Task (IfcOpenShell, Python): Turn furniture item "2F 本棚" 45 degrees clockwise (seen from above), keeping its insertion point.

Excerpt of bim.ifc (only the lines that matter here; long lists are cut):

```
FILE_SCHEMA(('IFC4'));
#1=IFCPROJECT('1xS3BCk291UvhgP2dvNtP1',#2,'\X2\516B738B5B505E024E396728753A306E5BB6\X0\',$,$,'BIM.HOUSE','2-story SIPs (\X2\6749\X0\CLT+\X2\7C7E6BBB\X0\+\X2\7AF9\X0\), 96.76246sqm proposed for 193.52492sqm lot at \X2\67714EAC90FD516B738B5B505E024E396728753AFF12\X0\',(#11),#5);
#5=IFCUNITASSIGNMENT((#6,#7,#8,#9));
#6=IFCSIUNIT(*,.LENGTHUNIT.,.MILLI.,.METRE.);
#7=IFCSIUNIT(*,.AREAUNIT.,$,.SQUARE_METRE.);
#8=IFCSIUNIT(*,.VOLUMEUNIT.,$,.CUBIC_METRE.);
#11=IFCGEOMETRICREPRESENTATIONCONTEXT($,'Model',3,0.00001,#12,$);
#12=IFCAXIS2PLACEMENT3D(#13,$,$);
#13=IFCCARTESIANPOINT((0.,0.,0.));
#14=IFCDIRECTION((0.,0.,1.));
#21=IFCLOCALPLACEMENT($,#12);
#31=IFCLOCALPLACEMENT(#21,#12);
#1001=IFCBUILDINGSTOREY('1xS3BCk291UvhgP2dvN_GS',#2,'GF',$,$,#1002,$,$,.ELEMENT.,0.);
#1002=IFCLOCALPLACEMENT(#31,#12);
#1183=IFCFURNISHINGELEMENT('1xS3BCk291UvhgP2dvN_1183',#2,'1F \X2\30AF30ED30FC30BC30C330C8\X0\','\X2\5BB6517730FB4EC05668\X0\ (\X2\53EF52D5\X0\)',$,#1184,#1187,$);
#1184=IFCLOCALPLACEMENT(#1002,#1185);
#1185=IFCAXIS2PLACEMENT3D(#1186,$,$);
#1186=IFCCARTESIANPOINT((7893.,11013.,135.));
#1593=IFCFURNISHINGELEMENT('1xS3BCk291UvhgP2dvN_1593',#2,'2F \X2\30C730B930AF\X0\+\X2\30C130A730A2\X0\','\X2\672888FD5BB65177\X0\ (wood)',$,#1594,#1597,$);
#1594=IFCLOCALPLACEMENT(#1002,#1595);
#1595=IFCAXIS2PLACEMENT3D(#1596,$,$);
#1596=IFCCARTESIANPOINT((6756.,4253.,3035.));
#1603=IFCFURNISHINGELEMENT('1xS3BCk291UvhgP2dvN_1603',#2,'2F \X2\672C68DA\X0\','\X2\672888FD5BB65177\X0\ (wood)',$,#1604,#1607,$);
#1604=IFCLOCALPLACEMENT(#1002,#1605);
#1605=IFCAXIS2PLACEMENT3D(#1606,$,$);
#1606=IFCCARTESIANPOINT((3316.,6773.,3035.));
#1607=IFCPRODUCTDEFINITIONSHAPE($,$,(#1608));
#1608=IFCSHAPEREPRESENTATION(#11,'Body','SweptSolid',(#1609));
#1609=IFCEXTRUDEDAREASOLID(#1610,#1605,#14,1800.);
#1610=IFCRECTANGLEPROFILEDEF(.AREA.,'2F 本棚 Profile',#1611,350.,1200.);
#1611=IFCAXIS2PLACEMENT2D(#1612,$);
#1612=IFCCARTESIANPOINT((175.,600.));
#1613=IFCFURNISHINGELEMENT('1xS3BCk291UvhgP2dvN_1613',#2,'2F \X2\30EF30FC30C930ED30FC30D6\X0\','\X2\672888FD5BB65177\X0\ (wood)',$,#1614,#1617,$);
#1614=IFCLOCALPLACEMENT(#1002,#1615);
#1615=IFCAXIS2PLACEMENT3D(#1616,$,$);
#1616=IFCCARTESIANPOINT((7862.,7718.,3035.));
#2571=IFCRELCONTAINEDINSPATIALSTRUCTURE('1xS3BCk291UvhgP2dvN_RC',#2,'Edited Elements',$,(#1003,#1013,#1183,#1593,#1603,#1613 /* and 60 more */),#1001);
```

```python
import ifcopenshell
import ifcopenshell.api.geometry
import ifcopenshell.util.placement

model = ifcopenshell.open("bim.ifc")

item = model.by_guid("1xS3BCk291UvhgP2dvN_1603")
matrix = ifcopenshell.util.placement.get_local_placement(item.ObjectPlacement)
matrix = matrix @ ifcopenshell.util.placement.rotation(-45, "Z")
ifcopenshell.api.geometry.edit_object_placement(model, product=item, matrix=matrix, is_si=False)

print(ifcopenshell.util.placement.get_local_placement(item.ObjectPlacement).round(3) + 0.0)

model.write("bim_rev.ifc")
```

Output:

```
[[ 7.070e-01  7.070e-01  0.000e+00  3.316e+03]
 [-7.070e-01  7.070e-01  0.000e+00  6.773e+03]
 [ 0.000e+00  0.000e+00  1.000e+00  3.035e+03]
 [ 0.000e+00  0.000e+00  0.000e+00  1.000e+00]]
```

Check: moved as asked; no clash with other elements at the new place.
